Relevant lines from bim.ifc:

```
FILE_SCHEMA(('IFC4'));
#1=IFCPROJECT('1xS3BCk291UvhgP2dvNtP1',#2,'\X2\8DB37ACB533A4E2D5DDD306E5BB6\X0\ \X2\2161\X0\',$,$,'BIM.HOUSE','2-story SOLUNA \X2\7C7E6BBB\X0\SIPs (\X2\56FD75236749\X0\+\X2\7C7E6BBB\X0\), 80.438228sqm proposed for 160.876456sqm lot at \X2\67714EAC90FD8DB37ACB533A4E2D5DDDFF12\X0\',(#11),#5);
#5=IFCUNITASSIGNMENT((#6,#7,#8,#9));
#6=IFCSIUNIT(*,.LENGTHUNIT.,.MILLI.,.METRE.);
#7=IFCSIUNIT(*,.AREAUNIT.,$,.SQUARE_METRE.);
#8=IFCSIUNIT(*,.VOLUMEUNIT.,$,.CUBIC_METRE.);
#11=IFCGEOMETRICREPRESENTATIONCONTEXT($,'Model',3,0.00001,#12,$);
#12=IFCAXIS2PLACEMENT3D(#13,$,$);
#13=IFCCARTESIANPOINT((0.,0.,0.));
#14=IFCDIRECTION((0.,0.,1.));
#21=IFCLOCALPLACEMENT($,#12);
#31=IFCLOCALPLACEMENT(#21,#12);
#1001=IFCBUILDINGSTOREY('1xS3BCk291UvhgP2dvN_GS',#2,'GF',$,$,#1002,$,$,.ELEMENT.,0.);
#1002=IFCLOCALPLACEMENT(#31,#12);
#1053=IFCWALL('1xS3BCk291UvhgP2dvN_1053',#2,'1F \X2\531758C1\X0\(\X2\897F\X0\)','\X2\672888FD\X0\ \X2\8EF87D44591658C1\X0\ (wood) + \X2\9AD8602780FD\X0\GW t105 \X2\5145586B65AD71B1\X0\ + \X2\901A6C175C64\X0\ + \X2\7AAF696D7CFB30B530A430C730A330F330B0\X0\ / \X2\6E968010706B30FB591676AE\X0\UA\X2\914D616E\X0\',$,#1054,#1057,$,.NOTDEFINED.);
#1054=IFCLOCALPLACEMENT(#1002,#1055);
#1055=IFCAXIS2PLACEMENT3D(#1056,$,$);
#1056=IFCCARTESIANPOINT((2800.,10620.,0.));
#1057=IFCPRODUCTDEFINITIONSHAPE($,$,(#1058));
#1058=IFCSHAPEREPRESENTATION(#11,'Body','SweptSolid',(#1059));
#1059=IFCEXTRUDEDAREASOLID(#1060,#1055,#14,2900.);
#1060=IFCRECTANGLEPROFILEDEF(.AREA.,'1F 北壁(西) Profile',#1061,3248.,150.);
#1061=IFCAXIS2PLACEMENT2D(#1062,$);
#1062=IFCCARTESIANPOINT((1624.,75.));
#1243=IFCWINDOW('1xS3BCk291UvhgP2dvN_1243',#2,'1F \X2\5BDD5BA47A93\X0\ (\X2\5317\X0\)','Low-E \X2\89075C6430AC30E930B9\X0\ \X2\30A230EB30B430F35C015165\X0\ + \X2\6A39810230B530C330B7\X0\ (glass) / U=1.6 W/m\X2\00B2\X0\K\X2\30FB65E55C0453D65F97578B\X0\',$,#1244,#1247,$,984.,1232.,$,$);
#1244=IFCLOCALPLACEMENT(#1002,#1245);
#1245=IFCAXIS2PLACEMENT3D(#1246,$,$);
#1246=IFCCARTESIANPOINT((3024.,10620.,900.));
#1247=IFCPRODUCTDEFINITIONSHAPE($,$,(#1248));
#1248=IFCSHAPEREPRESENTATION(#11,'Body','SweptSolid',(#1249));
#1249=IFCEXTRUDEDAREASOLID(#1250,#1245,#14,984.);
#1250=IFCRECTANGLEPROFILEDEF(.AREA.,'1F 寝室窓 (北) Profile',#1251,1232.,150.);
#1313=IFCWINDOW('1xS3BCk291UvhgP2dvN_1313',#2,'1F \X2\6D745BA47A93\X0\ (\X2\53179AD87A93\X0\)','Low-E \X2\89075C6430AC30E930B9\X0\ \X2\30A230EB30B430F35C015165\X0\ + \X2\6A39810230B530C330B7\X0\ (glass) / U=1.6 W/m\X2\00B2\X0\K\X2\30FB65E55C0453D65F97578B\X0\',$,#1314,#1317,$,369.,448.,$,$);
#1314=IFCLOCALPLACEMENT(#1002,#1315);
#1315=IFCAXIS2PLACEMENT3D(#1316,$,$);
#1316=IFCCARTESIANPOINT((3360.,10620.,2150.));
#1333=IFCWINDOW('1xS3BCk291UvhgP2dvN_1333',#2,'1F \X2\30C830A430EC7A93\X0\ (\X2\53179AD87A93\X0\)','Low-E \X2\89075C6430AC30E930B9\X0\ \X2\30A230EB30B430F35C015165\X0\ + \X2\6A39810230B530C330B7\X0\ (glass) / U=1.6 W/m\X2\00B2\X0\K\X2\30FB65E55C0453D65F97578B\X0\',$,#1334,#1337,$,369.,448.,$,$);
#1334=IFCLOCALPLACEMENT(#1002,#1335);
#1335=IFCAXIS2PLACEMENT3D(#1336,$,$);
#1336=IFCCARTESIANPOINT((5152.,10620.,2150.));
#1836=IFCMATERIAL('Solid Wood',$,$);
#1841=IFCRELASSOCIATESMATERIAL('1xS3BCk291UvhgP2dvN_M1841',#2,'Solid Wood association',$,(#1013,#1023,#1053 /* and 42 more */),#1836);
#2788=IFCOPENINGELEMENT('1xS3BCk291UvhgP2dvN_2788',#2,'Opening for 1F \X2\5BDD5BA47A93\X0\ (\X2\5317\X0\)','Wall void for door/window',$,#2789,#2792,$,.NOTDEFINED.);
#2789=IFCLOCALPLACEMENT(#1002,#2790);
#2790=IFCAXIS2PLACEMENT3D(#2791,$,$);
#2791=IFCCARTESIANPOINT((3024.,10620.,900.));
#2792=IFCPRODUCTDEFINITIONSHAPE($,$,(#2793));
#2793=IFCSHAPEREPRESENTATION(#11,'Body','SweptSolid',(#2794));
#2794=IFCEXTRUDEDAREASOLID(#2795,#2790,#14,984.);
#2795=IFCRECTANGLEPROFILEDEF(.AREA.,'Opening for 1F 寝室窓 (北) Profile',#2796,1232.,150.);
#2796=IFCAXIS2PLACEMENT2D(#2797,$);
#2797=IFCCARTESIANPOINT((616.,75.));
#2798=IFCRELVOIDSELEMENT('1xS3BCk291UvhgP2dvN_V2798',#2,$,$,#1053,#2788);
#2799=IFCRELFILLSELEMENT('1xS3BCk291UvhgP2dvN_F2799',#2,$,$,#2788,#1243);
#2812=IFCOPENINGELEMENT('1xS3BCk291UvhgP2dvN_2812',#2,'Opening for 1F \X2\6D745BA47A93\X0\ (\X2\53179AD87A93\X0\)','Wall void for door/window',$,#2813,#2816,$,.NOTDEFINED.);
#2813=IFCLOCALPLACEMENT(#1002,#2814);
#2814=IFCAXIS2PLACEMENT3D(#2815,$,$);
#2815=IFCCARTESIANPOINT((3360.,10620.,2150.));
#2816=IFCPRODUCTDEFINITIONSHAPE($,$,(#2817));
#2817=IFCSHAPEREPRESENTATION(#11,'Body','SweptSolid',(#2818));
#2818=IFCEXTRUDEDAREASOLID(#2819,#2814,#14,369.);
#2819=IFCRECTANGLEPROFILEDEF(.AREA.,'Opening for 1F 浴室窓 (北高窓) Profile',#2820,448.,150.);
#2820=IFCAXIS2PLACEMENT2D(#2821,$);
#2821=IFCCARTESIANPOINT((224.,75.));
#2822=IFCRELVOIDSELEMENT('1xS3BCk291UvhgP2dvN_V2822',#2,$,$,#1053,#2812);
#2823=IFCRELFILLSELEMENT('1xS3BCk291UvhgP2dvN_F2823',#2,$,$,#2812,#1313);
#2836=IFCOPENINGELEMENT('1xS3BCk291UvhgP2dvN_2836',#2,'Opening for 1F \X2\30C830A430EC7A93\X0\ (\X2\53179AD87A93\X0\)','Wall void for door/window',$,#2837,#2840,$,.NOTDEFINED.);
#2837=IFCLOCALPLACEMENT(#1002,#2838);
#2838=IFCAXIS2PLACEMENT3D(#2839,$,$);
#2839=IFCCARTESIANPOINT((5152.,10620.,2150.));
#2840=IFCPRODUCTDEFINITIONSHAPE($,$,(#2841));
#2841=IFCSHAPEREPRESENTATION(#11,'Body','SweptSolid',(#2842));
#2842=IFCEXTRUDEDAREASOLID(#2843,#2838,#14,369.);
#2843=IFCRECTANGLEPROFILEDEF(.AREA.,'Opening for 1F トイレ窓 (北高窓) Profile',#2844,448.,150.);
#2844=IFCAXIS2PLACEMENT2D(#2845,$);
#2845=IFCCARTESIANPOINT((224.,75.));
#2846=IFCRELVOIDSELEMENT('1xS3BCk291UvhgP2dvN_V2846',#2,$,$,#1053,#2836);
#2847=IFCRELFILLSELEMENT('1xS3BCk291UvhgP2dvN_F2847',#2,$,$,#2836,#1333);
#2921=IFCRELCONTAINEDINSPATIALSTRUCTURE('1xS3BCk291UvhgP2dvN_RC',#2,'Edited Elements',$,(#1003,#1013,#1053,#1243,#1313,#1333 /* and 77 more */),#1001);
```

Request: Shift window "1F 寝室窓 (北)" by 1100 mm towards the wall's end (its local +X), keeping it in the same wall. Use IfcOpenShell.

```python
import ifcopenshell
import ifcopenshell.api.geometry
import ifcopenshell.util.placement

model = ifcopenshell.open("bim.ifc")

window = model.by_id(1243)
opening = window.FillsVoids[0].RelatingOpeningElement
wall = opening.VoidsElements[0].RelatingBuildingElement

wall_matrix = ifcopenshell.util.placement.get_local_placement(wall.ObjectPlacement)
shift = wall_matrix[:3, 0] * 1100.0
before = ifcopenshell.util.placement.get_local_placement(window.ObjectPlacement)[:3, 3].copy()

# The window is not placed relative to its opening, so move both.
for product in (opening, window):
    matrix = ifcopenshell.util.placement.get_local_placement(product.ObjectPlacement)
    matrix[:3, 3] += shift
    ifcopenshell.api.geometry.edit_object_placement(model, product=product, matrix=matrix, is_si=False)

after = ifcopenshell.util.placement.get_local_placement(window.ObjectPlacement)[:3, 3]
print("window moved by", (after - before).round(3) + 0.0)

model.write("bim_rev.ifc")
```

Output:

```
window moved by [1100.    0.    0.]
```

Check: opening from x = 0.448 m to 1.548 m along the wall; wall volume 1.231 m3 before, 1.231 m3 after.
